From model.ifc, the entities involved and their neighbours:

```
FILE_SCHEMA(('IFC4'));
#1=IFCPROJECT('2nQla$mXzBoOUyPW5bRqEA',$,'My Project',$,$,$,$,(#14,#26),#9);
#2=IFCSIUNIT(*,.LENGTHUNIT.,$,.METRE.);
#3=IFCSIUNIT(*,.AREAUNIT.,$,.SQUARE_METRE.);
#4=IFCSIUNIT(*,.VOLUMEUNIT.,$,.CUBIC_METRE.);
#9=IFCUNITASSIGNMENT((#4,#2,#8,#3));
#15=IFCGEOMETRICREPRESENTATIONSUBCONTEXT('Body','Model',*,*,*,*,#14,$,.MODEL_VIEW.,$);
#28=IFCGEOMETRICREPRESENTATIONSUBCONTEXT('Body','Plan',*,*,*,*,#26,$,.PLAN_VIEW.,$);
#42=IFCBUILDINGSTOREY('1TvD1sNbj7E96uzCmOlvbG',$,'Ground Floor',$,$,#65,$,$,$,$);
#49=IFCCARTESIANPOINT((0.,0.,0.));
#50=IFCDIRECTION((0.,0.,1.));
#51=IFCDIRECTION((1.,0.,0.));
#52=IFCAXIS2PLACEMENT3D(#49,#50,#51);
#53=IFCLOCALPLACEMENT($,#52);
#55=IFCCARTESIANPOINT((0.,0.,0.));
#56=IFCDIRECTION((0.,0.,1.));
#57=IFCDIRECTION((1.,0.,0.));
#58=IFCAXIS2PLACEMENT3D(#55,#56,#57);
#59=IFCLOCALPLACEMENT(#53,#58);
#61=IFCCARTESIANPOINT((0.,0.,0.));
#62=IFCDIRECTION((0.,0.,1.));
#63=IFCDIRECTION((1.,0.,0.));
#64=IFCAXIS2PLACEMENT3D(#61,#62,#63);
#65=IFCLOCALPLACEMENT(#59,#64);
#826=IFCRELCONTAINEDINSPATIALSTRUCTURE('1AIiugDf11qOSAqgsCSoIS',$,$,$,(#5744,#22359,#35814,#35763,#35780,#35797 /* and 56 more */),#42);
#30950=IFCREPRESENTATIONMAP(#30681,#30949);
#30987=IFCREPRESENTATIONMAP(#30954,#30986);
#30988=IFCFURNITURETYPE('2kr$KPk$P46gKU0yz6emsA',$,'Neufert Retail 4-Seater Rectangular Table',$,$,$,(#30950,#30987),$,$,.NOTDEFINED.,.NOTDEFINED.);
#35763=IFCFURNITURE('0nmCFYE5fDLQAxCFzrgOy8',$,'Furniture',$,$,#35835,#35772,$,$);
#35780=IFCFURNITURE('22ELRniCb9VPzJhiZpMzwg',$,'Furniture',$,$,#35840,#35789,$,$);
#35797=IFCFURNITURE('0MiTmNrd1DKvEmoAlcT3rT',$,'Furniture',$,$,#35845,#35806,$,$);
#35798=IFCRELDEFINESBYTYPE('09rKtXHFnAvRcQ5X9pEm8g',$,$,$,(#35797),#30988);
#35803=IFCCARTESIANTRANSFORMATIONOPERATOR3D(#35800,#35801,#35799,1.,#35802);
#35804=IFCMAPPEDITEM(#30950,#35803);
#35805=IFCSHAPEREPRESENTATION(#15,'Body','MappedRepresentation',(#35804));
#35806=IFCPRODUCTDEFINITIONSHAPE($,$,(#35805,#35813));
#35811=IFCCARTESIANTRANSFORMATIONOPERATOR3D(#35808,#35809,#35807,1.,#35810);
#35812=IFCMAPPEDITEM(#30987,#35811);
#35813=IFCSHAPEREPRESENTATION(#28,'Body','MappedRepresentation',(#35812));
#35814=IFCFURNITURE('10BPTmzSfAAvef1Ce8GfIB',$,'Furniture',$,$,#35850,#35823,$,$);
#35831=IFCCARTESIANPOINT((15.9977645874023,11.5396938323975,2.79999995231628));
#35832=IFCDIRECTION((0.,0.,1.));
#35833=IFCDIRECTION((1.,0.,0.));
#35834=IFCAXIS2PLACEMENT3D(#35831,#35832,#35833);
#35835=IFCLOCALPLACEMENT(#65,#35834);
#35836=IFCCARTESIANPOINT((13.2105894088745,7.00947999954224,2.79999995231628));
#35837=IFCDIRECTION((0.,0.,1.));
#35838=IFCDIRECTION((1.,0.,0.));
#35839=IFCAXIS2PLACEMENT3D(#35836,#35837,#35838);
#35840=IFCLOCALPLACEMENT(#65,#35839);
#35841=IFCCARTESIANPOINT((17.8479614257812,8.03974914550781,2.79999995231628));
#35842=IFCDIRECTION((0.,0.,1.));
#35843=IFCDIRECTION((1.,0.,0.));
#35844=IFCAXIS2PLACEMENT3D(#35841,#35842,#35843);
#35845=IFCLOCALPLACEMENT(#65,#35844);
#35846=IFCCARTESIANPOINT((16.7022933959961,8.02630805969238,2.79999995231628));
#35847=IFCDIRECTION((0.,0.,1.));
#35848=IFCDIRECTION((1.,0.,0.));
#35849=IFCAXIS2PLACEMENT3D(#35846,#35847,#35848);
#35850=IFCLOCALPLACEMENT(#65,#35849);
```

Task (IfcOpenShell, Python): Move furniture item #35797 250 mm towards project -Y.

```python
import ifcopenshell
import ifcopenshell.api.geometry
import ifcopenshell.util.placement
import ifcopenshell.util.unit

model = ifcopenshell.open("model.ifc")
unit_scale = ifcopenshell.util.unit.calculate_unit_scale(model)

item = model.by_guid("0MiTmNrd1DKvEmoAlcT3rT")
matrix = ifcopenshell.util.placement.get_local_placement(item.ObjectPlacement)
matrix[1, 3] -= 0.25 / unit_scale
ifcopenshell.api.geometry.edit_object_placement(model, product=item, matrix=matrix, is_si=False)

print(ifcopenshell.util.placement.get_local_placement(item.ObjectPlacement).round(3) + 0.0)

model.write("model_rev.ifc")
```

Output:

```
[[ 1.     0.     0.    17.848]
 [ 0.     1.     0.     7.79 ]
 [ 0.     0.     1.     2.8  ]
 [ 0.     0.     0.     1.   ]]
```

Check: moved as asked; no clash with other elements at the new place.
